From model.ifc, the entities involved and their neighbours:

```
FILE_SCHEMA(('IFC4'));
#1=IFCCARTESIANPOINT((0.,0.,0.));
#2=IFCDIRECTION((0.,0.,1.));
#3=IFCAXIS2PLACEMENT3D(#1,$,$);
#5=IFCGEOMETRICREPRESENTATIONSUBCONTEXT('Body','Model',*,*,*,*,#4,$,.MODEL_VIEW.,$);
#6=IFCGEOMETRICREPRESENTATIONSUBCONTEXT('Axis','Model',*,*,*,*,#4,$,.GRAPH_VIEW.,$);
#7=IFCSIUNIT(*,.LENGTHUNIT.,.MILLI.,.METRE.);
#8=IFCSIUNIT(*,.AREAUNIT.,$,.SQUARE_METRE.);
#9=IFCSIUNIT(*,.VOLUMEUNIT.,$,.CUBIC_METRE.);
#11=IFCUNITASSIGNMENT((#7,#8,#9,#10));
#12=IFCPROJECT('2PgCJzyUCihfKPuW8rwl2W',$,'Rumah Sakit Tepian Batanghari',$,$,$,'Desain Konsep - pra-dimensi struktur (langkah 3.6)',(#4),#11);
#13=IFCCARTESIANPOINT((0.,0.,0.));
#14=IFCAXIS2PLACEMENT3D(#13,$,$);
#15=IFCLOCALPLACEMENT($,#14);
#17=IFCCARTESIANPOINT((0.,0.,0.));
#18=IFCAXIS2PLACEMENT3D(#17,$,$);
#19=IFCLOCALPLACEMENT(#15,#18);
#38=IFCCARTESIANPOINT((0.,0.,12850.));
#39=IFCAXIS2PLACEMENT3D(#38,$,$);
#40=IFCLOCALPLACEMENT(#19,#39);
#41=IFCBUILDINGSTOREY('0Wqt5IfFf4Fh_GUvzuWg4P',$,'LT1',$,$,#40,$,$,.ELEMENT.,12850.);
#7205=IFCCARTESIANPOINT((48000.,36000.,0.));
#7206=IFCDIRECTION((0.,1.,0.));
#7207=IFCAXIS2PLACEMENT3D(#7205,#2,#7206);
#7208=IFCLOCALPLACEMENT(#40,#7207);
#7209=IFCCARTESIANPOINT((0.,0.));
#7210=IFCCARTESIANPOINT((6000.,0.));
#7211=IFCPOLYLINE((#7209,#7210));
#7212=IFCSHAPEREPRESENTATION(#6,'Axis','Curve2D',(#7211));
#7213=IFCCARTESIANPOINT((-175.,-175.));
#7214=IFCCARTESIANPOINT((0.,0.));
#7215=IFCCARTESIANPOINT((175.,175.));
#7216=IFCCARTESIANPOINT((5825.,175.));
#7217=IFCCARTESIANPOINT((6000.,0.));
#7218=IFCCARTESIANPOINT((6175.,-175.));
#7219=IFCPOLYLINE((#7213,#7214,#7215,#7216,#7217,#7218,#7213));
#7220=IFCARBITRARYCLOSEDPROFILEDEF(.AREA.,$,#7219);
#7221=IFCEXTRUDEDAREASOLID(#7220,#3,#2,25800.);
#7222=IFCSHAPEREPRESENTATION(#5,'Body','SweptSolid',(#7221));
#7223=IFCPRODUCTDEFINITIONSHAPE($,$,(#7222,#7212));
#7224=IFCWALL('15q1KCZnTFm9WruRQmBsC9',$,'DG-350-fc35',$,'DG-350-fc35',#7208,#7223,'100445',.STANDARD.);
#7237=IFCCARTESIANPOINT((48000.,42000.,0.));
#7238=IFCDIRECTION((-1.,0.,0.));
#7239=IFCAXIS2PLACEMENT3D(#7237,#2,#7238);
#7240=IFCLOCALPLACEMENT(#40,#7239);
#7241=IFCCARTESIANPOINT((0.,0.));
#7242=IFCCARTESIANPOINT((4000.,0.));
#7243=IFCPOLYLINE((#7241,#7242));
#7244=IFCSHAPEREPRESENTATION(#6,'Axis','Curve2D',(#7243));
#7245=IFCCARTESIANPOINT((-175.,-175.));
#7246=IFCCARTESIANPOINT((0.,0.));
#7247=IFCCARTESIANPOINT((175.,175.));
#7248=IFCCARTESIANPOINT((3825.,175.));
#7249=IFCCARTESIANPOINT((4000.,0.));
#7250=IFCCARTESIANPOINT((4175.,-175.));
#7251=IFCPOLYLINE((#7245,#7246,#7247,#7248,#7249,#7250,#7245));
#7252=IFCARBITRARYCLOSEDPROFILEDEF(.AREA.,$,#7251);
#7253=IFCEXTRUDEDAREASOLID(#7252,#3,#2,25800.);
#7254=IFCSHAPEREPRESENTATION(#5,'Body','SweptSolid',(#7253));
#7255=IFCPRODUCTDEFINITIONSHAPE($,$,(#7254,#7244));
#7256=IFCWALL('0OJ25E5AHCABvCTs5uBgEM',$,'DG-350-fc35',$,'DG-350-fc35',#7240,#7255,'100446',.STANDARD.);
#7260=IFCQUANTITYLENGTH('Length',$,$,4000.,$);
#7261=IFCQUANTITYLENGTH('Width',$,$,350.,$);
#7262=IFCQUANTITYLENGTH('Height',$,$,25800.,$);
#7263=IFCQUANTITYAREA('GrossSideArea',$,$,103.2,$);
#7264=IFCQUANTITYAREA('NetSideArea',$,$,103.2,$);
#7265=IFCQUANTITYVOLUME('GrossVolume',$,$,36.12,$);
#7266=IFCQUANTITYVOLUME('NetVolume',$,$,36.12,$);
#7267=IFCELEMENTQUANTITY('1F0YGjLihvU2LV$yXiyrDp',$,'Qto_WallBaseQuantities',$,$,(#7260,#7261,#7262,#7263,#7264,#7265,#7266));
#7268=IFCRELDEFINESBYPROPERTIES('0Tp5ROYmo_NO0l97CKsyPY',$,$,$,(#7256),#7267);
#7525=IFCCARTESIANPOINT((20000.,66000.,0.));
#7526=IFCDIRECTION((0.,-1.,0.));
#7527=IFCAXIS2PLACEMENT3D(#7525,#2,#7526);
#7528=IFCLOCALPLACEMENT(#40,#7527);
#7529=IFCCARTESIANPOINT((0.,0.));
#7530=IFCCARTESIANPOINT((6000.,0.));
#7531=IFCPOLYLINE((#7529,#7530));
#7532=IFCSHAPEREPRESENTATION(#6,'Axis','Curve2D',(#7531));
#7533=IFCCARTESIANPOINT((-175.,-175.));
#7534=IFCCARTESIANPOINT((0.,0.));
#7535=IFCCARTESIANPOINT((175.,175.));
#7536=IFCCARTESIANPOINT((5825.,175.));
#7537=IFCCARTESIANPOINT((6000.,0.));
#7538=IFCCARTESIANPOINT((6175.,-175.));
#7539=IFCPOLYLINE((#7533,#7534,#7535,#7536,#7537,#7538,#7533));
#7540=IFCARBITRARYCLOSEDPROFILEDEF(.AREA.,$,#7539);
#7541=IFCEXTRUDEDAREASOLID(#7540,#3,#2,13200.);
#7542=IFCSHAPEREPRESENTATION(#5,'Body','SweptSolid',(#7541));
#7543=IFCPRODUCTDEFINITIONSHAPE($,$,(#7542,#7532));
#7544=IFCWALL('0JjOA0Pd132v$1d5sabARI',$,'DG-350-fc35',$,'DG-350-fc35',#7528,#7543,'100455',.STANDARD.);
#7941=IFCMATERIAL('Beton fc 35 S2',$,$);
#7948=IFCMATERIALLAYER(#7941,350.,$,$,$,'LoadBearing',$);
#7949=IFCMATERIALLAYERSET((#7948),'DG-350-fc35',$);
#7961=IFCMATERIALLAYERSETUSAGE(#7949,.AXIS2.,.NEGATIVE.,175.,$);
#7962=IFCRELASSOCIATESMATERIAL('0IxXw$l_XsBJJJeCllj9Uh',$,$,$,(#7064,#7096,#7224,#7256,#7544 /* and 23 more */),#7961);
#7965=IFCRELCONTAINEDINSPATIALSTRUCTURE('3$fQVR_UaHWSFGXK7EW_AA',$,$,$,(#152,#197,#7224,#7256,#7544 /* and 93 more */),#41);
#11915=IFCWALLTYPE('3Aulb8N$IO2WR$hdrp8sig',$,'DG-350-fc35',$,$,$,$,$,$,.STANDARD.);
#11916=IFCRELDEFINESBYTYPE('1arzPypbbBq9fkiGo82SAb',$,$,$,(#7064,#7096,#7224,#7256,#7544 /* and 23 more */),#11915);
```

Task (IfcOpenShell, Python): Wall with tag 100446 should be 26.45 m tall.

```python
import ifcopenshell
import ifcopenshell.api.pset
import ifcopenshell.geom
import ifcopenshell.util.element
import ifcopenshell.util.representation
import ifcopenshell.util.shape
import ifcopenshell.util.unit

model = ifcopenshell.open("model.ifc")
unit_scale = ifcopenshell.util.unit.calculate_unit_scale(model)
area_scale = ifcopenshell.util.unit.calculate_unit_scale(model, "AREAUNIT")
volume_scale = ifcopenshell.util.unit.calculate_unit_scale(model, "VOLUMEUNIT")
settings = ifcopenshell.geom.settings()


def volume(element):
    """Net volume in cubic metres, openings subtracted."""
    shape = ifcopenshell.geom.create_shape(settings, element)
    return ifcopenshell.util.shape.get_volume(shape.geometry)


wall = model.by_guid("0OJ25E5AHCABvCTs5uBgEM")
before = volume(wall)

body = ifcopenshell.util.representation.get_representation(wall, "Model", "Body")
solid = body.Items[0]
old_height = solid.Depth
solid.Depth = 26.45 / unit_scale
after = volume(wall)
thickness = 0.35  # wall thickness in metres

# Update the stored height, areas and volumes.
qto = model.by_id(ifcopenshell.util.element.get_pset(wall, "Qto_WallBaseQuantities", should_inherit=False)["id"])
ifcopenshell.api.pset.edit_qto(model, qto=qto, properties={
    "Height": solid.Depth,
    "GrossSideArea": ifcopenshell.util.element.get_pset(wall, "Qto_WallBaseQuantities", "GrossSideArea") * solid.Depth / old_height,
    "NetSideArea": after / thickness / area_scale,
    "GrossVolume": ifcopenshell.util.element.get_pset(wall, "Qto_WallBaseQuantities", "GrossVolume") * solid.Depth / old_height,
    "NetVolume": after / volume_scale,
})

print(f"height {old_height:g} -> {solid.Depth:g}, volume {before:.3f} -> {after:.3f} m3")

model.write("model_v2.ifc")
```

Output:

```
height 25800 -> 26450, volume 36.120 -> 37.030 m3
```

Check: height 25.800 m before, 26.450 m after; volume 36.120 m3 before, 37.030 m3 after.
